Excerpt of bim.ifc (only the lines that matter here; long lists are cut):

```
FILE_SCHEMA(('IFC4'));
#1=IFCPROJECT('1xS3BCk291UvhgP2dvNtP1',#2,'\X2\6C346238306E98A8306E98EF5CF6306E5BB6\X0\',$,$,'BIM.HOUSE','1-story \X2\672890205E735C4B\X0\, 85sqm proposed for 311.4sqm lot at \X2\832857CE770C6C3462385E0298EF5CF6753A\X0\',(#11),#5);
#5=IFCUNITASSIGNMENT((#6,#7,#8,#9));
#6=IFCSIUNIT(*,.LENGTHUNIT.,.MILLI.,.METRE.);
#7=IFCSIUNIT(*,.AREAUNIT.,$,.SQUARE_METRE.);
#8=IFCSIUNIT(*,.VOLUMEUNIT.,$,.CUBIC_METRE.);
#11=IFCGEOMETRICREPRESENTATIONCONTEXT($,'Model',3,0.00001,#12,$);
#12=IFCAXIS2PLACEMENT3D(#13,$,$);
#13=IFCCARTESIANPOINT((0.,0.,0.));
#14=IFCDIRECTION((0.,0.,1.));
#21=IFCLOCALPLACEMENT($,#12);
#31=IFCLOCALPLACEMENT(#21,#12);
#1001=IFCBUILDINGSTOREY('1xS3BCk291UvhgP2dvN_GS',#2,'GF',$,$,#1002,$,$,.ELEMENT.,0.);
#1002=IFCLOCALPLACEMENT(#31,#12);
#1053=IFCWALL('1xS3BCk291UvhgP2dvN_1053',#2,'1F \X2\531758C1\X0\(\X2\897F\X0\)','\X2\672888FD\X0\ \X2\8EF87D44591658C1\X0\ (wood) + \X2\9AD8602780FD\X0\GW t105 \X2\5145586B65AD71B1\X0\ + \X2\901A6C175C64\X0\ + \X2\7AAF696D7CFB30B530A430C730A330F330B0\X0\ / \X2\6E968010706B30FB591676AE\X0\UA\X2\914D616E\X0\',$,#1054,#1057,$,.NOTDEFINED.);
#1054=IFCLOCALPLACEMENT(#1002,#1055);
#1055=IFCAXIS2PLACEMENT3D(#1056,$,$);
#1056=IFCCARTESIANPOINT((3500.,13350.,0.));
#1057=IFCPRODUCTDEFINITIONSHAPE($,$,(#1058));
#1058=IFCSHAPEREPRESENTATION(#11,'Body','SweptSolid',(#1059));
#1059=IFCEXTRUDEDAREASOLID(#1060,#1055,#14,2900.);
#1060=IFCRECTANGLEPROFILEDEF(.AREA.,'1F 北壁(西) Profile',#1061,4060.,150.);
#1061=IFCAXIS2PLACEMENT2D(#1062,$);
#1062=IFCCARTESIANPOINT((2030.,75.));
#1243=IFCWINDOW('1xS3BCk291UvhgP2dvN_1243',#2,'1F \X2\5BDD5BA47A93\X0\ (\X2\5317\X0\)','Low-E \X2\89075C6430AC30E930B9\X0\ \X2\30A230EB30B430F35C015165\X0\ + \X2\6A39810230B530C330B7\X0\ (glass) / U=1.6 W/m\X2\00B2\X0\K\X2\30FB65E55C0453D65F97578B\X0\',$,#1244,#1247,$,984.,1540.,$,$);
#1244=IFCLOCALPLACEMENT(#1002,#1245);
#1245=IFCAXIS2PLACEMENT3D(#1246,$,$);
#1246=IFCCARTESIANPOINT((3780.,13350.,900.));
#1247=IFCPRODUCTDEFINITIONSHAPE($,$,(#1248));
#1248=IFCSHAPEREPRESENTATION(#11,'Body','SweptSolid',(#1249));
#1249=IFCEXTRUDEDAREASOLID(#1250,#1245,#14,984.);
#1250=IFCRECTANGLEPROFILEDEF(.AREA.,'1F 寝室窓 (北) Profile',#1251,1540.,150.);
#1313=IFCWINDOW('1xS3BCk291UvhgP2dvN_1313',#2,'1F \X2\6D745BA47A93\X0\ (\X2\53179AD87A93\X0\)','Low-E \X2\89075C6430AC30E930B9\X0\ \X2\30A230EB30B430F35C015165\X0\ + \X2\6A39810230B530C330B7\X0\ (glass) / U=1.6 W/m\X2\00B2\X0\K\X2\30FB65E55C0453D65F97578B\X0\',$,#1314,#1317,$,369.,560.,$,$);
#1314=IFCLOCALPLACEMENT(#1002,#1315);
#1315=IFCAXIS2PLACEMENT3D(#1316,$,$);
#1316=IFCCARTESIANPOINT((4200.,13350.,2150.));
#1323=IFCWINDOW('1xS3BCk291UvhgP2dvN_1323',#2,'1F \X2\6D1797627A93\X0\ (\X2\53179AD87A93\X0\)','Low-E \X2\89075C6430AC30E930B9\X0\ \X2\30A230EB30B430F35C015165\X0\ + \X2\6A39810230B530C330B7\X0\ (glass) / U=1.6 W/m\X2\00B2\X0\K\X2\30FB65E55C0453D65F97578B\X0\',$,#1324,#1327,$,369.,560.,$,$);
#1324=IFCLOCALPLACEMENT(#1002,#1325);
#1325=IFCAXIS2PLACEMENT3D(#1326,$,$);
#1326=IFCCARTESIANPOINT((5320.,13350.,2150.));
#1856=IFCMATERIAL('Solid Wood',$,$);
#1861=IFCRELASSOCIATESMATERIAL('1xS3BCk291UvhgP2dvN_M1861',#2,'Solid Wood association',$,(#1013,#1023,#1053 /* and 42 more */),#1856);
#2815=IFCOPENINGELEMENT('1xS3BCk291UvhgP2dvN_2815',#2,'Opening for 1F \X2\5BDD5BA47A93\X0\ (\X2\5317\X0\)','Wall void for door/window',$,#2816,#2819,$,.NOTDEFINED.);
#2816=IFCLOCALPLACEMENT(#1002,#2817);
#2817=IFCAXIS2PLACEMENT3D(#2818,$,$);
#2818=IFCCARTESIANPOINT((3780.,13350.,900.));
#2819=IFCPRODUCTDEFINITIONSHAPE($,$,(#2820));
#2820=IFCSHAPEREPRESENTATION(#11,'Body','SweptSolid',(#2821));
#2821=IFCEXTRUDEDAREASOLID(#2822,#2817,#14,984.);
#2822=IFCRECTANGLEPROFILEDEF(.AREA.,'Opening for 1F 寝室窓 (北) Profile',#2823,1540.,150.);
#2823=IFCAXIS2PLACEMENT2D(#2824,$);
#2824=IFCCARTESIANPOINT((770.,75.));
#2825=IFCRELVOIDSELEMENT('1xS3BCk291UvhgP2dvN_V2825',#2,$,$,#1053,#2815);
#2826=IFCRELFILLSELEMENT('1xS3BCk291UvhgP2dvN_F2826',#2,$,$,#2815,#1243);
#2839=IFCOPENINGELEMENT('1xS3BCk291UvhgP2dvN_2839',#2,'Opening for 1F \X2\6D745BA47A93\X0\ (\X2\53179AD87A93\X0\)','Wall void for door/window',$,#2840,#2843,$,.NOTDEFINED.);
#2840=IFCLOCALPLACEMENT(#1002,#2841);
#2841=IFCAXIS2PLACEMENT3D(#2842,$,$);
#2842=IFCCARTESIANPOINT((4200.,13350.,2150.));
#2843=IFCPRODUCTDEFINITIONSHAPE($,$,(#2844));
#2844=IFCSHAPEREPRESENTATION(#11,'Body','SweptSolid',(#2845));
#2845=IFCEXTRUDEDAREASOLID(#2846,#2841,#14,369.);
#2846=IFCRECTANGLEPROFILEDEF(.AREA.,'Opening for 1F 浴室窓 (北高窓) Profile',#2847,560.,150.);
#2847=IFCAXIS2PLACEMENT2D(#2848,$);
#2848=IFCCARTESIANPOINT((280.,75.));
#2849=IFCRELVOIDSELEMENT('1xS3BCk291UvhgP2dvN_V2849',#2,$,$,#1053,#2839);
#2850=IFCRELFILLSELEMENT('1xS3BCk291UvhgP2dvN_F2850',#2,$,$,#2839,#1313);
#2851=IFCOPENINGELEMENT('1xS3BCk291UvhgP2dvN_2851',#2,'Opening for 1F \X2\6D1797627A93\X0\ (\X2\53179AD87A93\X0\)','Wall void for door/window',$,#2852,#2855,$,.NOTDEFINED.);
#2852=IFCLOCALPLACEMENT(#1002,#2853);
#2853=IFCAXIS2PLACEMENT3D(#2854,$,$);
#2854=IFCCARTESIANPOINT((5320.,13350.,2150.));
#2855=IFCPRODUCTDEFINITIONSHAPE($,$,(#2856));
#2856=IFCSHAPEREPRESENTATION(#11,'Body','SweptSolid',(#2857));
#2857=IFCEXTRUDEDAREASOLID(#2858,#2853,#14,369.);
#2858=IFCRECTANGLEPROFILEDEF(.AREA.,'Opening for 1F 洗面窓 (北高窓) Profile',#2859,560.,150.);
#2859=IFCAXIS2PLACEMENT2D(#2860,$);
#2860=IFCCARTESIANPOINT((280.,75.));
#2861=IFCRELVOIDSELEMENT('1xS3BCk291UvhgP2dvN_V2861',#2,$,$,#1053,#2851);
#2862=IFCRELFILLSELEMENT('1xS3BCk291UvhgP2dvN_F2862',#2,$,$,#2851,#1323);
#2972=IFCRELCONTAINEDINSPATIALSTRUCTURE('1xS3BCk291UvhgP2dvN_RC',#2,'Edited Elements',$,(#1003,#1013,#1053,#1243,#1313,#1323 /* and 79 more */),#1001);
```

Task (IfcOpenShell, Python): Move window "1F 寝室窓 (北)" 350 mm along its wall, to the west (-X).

```python
import ifcopenshell
import ifcopenshell.api.geometry
import ifcopenshell.util.placement
import ifcopenshell.util.unit

model = ifcopenshell.open("bim.ifc")
unit_scale = ifcopenshell.util.unit.calculate_unit_scale(model)

window = model.by_guid("1xS3BCk291UvhgP2dvN_1243")
opening = window.FillsVoids[0].RelatingOpeningElement
wall = opening.VoidsElements[0].RelatingBuildingElement

wall_matrix = ifcopenshell.util.placement.get_local_placement(wall.ObjectPlacement)
shift = wall_matrix[:3, 0] * -0.35 / unit_scale
before = ifcopenshell.util.placement.get_local_placement(window.ObjectPlacement)[:3, 3].copy()

# The window is not placed relative to its opening, so move both.
for product in (opening, window):
    matrix = ifcopenshell.util.placement.get_local_placement(product.ObjectPlacement)
    matrix[:3, 3] += shift
    ifcopenshell.api.geometry.edit_object_placement(model, product=product, matrix=matrix, is_si=False)

after = ifcopenshell.util.placement.get_local_placement(window.ObjectPlacement)[:3, 3]
print("window moved by", (after - before).round(3) + 0.0)

model.write("bim_rev.ifc")
```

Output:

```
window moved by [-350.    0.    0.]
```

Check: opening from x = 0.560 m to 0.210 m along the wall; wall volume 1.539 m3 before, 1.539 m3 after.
